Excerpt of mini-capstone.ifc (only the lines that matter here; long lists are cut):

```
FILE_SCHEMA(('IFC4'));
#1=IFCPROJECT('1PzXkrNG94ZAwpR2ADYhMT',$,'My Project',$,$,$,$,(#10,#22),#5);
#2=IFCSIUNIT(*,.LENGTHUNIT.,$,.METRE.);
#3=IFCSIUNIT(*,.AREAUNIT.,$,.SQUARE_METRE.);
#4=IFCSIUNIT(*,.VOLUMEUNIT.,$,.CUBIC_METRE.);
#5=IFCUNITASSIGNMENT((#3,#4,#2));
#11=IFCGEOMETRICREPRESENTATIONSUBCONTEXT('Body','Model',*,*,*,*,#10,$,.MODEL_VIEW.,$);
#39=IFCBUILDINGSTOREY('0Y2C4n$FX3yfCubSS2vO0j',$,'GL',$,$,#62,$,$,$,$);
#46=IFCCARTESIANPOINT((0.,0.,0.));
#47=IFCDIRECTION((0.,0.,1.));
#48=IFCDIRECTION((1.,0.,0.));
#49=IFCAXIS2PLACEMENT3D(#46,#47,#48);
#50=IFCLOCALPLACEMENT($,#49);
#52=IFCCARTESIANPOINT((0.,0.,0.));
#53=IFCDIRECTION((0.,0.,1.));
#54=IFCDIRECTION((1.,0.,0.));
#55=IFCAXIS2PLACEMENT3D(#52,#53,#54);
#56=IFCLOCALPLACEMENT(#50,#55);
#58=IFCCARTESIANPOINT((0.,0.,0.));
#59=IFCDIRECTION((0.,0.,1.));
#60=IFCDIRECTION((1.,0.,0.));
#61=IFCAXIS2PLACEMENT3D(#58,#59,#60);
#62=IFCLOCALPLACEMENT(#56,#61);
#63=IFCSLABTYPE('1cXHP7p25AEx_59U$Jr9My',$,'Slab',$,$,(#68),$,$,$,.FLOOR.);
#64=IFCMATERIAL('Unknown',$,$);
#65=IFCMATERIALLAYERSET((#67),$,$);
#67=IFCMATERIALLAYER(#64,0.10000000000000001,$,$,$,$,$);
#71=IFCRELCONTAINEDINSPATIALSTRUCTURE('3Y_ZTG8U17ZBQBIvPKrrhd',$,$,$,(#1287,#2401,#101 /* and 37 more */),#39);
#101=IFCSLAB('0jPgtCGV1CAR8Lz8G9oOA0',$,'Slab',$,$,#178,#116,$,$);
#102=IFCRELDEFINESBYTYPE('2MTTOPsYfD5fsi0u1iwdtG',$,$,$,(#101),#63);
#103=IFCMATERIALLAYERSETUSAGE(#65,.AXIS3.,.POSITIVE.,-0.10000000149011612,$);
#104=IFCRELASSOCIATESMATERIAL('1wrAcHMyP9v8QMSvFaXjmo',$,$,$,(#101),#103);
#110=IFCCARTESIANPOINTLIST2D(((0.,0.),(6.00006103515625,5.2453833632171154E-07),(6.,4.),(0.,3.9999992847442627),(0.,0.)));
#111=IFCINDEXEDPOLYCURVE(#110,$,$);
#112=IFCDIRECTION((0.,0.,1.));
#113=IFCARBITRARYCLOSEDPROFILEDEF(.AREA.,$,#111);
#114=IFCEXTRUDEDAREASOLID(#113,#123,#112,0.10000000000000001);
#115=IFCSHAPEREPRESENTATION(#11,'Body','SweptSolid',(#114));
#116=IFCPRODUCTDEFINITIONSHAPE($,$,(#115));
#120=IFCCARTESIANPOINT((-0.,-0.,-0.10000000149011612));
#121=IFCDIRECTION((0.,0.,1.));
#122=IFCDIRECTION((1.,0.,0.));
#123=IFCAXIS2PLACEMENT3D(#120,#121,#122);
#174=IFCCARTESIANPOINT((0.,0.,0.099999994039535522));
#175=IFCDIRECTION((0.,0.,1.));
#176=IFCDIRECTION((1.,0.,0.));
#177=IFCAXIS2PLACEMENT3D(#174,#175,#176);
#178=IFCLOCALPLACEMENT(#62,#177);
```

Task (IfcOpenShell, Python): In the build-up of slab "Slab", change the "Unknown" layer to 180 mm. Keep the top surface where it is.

```python
import ifcopenshell
import ifcopenshell.util.element
import ifcopenshell.util.representation

model = ifcopenshell.open("mini-capstone.ifc")

layer_set = model.by_id(65)
layer = next(l for l in layer_set.MaterialLayers if l.Material and l.Material.Name == "Unknown")
change = 0.18 - layer.LayerThickness
layer.LayerThickness += change

# Geometry does not follow the layer set by itself.
slabs = [e for e in ifcopenshell.util.element.get_elements_by_material(model, layer_set) if e.is_a("IfcSlab")]
for slab in sorted(slabs, key=lambda e: e.id()):
    body = ifcopenshell.util.representation.get_representation(slab, "Model", "Body")
    solid = body.Items[0]
    old_depth = solid.Depth
    solid.Depth += change
    # Extruded upwards: lower the start of the extrusion so the top stays.
    x, y, z = solid.Position.Location.Coordinates
    solid.Position.Location = model.createIfcCartesianPoint((x, y, z - change))
    print(slab.id(), f"{old_depth:g} -> {solid.Depth:g}")

# The layers are counted up from the underside, which has moved.
for usage in {ifcopenshell.util.element.get_material(slab) for slab in slabs}:
    usage.OffsetFromReferenceLine -= change

model.write("mini-capstone_updated.ifc")
```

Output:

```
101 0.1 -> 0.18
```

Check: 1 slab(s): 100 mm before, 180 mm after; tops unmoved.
